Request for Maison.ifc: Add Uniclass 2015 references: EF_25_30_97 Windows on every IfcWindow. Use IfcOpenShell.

First a look at what the model holds.

```python
import ifcopenshell

model = ifcopenshell.open("Maison.ifc")
print(model.schema)
print("classifications:", [c.Name for c in model.by_type("IfcClassification")])
for ifc_class in ("IfcDoor", "IfcRoof", "IfcStair", "IfcWall", "IfcWindow"):
    print(ifc_class, len(model.by_type(ifc_class)))
```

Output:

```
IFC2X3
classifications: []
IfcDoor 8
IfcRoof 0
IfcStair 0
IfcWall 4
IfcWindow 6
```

```python
import ifcopenshell
import ifcopenshell.api.classification

model = ifcopenshell.open("Maison.ifc")

# IFC2X3 requires Source and Edition and has no link from the project to the system.
system = model.create_entity("IfcClassification", Source="NBS", Edition="2015", Name="Uniclass 2015")

codes = {
    "IfcWindow": ("EF_25_30_97", "Windows"),
}
for ifc_class, (code, name) in codes.items():
    products = model.by_type(ifc_class)
    ifcopenshell.api.classification.add_reference(
        model, products=products, classification=system, identification=code, name=name
    )
    print(code, len(products))

model.write("Maison_v2.ifc")
```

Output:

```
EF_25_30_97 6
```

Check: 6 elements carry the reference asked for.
